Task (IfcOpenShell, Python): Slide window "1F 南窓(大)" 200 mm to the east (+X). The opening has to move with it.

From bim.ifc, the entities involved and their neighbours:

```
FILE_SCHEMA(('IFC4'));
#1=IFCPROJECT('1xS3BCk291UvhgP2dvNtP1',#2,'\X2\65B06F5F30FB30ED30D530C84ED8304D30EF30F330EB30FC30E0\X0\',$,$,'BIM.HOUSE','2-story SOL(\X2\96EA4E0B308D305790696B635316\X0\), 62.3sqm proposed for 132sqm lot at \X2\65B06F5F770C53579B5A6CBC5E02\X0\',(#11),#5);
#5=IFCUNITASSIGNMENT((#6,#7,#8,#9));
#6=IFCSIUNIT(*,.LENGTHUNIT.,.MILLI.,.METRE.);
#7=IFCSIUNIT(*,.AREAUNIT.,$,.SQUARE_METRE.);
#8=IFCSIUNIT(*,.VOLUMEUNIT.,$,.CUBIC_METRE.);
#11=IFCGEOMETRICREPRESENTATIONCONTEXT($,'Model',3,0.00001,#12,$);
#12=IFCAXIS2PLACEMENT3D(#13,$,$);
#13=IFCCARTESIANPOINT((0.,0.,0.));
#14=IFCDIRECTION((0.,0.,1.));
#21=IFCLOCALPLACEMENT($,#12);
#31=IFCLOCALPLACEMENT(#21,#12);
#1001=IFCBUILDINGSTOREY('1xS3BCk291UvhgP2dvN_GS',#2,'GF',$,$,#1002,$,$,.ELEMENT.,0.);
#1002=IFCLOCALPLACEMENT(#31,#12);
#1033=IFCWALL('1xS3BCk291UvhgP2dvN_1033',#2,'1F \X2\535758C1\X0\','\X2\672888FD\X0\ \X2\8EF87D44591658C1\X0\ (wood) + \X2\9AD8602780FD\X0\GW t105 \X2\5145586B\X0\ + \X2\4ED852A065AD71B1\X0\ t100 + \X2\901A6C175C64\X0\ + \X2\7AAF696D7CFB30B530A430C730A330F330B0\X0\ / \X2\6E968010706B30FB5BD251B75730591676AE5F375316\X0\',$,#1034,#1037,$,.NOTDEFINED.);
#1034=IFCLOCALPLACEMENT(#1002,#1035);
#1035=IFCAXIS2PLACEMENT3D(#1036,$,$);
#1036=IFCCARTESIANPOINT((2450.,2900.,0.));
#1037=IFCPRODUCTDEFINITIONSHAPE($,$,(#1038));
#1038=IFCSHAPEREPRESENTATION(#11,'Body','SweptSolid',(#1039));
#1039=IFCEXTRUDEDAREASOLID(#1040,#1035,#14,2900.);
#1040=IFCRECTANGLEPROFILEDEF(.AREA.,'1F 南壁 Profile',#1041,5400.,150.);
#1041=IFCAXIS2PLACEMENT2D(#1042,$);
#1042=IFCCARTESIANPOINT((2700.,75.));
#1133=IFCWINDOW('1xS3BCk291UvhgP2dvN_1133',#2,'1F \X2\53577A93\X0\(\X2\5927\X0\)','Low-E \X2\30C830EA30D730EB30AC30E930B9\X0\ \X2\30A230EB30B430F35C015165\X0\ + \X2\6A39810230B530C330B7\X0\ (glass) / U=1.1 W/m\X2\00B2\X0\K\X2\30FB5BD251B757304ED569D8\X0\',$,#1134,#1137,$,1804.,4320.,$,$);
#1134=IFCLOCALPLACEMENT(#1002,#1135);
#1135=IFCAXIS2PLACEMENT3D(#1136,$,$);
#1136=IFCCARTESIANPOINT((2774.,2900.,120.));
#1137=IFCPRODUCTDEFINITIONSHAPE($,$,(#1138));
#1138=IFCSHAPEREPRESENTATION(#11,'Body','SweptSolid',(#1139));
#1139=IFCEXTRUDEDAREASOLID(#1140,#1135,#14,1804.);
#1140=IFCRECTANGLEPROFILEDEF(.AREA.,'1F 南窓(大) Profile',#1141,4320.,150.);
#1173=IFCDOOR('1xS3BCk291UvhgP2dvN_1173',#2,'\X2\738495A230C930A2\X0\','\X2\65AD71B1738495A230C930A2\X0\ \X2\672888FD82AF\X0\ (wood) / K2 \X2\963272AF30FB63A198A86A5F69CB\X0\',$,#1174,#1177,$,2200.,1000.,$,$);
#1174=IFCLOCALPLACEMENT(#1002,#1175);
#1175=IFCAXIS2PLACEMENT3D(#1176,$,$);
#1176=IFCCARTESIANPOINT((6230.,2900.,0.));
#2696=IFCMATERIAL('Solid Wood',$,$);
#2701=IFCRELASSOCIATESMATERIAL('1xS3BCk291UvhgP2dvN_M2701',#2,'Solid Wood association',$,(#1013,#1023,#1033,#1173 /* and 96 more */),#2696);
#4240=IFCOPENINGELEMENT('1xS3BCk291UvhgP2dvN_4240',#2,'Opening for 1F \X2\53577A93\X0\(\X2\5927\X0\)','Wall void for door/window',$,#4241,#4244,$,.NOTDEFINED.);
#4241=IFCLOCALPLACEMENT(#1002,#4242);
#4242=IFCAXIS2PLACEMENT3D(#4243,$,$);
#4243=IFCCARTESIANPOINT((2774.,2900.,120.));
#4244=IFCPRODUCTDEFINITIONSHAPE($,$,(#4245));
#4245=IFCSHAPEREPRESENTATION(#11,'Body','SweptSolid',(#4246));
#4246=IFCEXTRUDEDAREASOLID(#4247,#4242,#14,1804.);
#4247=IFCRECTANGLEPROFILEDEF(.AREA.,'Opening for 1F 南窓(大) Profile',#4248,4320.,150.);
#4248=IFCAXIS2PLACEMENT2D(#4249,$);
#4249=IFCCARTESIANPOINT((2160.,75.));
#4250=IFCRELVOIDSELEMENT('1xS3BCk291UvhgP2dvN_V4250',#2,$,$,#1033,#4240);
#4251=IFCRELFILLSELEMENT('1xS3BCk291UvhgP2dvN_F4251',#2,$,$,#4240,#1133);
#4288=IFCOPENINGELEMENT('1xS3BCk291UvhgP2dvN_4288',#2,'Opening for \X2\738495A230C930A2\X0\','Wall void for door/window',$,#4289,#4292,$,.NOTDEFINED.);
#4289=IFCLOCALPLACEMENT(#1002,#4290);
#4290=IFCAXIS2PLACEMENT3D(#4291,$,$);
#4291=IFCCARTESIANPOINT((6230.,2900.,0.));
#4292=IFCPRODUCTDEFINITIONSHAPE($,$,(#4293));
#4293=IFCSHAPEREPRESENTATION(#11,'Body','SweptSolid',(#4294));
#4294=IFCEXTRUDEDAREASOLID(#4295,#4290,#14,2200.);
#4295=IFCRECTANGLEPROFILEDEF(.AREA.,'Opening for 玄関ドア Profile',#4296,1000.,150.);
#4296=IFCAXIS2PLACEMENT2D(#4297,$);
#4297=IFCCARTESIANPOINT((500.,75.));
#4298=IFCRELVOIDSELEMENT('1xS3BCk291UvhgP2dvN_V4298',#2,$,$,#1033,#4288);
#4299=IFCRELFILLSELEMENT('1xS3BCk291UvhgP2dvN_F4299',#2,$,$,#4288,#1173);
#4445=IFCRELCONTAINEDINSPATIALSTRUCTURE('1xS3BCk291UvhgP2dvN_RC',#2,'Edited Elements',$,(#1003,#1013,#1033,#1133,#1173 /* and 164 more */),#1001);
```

```python
import ifcopenshell
import ifcopenshell.api.geometry
import ifcopenshell.util.placement
import ifcopenshell.util.unit

model = ifcopenshell.open("bim.ifc")
unit_scale = ifcopenshell.util.unit.calculate_unit_scale(model)

window = model.by_id(1133)
opening = window.FillsVoids[0].RelatingOpeningElement
wall = opening.VoidsElements[0].RelatingBuildingElement

wall_matrix = ifcopenshell.util.placement.get_local_placement(wall.ObjectPlacement)
shift = wall_matrix[:3, 0] * 0.2 / unit_scale
before = ifcopenshell.util.placement.get_local_placement(window.ObjectPlacement)[:3, 3].copy()

# The window is not placed relative to its opening, so move both.
for product in (opening, window):
    matrix = ifcopenshell.util.placement.get_local_placement(product.ObjectPlacement)
    matrix[:3, 3] += shift
    ifcopenshell.api.geometry.edit_object_placement(model, product=product, matrix=matrix, is_si=False)

after = ifcopenshell.util.placement.get_local_placement(window.ObjectPlacement)[:3, 3]
print("window moved by", (after - before).round(3) + 0.0)

model.write("bim_edited.ifc")
```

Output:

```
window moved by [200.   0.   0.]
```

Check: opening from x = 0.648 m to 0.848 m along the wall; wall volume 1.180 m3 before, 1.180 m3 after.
